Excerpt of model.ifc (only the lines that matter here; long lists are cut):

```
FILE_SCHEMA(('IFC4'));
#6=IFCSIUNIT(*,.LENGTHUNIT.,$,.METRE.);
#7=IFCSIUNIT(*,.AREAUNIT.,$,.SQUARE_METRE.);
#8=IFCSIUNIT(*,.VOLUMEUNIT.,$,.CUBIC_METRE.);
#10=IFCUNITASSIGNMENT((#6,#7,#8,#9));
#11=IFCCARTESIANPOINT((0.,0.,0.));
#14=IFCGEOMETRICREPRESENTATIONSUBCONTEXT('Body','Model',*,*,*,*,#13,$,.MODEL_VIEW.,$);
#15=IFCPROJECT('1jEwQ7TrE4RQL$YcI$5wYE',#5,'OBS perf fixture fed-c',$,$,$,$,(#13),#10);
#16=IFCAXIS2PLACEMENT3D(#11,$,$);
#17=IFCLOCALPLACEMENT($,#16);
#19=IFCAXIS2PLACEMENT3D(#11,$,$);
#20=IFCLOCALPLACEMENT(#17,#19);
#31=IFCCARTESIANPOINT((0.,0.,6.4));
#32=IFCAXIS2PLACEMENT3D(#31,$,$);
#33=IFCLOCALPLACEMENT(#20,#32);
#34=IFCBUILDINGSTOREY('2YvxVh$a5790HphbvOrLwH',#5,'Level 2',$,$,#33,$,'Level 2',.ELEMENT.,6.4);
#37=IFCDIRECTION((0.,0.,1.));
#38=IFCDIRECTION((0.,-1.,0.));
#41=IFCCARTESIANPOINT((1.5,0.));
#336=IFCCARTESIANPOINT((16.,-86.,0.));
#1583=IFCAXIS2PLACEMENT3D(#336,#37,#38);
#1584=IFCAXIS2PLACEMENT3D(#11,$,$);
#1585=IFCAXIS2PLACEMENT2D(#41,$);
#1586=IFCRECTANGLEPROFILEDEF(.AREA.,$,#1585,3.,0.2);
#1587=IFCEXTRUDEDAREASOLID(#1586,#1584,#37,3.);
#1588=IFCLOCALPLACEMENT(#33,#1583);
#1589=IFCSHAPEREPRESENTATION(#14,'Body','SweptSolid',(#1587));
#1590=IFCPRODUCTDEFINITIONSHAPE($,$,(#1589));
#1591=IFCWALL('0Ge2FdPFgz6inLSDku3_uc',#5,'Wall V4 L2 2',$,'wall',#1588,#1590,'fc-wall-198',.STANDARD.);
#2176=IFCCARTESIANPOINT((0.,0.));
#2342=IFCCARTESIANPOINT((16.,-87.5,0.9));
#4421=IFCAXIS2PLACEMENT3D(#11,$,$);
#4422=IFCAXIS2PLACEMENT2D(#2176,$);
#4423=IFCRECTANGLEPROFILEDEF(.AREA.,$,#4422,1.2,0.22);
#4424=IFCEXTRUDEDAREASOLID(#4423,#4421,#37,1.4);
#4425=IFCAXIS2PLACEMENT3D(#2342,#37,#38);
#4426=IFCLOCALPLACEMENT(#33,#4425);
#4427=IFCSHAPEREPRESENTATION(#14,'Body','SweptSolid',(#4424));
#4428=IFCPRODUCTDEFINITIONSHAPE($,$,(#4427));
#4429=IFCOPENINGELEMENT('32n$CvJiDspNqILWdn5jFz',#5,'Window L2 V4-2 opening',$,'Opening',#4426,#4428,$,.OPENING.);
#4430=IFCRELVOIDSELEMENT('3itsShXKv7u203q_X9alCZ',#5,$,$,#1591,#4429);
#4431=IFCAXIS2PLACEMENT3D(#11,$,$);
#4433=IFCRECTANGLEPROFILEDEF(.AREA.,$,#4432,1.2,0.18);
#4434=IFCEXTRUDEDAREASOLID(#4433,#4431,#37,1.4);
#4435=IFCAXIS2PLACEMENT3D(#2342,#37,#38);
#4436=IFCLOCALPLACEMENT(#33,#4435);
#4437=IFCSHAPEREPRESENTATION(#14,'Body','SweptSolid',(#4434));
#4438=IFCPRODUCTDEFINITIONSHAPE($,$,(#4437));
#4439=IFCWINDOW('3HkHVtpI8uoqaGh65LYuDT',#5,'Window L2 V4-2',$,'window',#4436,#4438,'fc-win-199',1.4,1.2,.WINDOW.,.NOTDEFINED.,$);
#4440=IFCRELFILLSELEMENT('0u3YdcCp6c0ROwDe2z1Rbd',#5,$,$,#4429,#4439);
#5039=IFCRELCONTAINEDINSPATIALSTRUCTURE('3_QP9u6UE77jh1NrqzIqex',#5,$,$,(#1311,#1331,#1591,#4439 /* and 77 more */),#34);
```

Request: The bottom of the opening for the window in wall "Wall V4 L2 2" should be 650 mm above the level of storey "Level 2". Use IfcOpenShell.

```python
import numpy as np
import ifcopenshell
import ifcopenshell.api.geometry
import ifcopenshell.geom
import ifcopenshell.util.element
import ifcopenshell.util.placement
import ifcopenshell.util.shape
import ifcopenshell.util.unit

model = ifcopenshell.open("model.ifc")
unit_scale = ifcopenshell.util.unit.calculate_unit_scale(model)

window = model.by_guid("3HkHVtpI8uoqaGh65LYuDT")
opening = window.FillsVoids[0].RelatingOpeningElement
storey = ifcopenshell.util.element.get_container(window, ifc_class="IfcBuildingStorey")
level = ifcopenshell.util.placement.get_local_placement(storey.ObjectPlacement)[2, 3]

# The opening's origin need not be at the sill, so measure its lowest point.
shape = ifcopenshell.geom.create_shape(ifcopenshell.geom.settings(), opening)
bottom = ifcopenshell.util.shape.get_shape_bottom_elevation(shape, shape.geometry) / unit_scale
dz = level + 0.65 / unit_scale - bottom

shift = np.array([0.0, 0.0, dz])
# The window is not placed relative to its opening, so move both.
for product in (opening, window):
    matrix = ifcopenshell.util.placement.get_local_placement(product.ObjectPlacement)
    matrix[:3, 3] += shift
    ifcopenshell.api.geometry.edit_object_placement(model, product=product, matrix=matrix, is_si=False)

print(f"moved by {dz * unit_scale:+.3f} m")

model.write("model_updated.ifc")
```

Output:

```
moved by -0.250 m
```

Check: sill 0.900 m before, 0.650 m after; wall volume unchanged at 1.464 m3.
